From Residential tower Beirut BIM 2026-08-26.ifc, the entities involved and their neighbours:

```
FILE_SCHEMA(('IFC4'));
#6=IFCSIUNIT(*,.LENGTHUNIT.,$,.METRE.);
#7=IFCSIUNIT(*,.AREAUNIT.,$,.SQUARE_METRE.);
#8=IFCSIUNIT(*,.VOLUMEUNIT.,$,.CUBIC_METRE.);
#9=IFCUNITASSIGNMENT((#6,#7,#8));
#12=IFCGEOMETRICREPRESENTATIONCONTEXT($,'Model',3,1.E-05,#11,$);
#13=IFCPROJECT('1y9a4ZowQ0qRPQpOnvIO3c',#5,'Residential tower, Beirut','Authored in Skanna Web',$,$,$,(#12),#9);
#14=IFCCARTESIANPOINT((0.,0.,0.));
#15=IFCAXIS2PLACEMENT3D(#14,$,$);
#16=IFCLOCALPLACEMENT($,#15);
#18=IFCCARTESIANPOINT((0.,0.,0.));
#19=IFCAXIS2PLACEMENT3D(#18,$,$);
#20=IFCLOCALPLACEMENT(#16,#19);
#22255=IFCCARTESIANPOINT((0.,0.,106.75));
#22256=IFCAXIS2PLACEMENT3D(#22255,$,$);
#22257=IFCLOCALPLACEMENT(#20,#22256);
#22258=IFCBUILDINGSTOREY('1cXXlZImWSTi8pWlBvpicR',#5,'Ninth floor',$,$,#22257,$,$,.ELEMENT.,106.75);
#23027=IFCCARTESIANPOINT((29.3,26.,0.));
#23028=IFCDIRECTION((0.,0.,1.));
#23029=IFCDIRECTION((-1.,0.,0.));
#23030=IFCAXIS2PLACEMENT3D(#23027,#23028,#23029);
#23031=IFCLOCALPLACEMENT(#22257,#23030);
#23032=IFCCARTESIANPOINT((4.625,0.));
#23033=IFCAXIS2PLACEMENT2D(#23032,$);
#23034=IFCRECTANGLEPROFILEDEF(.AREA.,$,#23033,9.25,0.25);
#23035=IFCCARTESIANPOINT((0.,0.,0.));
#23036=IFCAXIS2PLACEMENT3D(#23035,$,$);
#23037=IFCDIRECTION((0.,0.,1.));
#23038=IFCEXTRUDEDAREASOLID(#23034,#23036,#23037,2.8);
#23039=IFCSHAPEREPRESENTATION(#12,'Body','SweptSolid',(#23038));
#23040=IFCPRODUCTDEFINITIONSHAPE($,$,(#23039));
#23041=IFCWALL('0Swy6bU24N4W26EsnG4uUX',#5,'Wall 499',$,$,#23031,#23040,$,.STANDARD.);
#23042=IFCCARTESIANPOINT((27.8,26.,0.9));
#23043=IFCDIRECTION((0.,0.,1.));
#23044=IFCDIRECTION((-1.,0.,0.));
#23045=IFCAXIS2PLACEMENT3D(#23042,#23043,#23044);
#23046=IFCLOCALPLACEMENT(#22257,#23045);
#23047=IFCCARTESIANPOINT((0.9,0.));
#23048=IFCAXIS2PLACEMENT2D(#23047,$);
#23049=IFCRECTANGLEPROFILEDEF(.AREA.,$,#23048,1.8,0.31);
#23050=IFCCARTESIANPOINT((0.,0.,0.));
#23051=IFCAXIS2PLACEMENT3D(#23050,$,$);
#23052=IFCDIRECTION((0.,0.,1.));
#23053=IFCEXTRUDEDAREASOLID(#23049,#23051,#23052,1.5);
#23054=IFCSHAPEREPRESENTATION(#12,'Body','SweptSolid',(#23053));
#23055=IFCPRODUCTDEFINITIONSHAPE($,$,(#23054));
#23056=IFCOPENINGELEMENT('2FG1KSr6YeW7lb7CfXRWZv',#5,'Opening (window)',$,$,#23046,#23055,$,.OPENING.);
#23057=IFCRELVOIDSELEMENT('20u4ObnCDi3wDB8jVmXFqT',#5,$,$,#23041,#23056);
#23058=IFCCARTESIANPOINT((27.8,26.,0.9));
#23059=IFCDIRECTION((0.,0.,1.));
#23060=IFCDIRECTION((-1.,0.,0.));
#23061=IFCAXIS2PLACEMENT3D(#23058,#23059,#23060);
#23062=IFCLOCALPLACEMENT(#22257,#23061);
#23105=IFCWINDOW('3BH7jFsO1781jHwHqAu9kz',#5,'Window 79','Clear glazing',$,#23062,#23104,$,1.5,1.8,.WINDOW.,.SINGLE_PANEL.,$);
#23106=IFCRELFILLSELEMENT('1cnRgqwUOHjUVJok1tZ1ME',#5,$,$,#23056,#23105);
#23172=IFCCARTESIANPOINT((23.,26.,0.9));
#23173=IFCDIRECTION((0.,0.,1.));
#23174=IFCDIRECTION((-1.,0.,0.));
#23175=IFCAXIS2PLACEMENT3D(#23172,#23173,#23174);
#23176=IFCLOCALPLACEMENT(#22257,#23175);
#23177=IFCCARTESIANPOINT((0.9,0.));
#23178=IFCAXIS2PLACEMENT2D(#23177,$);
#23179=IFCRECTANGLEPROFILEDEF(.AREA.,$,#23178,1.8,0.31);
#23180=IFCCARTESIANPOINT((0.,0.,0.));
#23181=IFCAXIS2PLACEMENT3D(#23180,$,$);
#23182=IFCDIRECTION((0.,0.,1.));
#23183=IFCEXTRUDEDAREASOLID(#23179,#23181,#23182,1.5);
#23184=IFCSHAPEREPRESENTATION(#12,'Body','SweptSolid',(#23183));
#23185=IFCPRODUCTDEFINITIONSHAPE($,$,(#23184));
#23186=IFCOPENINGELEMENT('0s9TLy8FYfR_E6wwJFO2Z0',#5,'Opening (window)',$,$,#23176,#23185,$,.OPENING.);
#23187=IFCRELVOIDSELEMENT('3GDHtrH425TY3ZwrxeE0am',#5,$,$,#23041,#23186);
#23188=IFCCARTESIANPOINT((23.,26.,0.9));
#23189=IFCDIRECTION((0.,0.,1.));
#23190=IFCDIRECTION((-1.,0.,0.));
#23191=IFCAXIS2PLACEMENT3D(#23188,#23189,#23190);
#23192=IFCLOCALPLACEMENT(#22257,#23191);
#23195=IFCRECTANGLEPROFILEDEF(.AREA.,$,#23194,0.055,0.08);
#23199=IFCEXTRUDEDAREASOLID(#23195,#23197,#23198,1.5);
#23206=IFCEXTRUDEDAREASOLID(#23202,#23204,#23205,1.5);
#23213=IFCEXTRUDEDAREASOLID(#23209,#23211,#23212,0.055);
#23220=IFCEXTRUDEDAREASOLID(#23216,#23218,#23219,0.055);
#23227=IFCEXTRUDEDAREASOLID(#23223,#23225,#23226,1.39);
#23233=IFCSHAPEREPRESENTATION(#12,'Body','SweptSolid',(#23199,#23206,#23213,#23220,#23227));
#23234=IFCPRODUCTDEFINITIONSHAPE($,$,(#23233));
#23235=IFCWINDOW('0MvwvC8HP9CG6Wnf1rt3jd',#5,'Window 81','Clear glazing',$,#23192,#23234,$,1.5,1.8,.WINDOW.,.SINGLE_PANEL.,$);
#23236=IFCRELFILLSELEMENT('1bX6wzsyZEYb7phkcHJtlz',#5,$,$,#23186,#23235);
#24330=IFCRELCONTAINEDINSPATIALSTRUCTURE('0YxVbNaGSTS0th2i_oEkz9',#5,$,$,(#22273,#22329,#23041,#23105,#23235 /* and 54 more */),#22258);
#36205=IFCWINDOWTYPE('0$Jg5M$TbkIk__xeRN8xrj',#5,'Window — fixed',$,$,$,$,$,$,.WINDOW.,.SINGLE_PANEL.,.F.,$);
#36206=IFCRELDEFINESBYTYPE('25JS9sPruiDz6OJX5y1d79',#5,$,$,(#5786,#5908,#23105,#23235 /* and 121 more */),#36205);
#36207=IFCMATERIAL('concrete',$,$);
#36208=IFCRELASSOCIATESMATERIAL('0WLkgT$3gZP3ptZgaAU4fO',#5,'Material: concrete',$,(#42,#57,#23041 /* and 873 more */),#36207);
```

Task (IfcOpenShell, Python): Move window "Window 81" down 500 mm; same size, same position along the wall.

```python
import numpy as np
import ifcopenshell
import ifcopenshell.api.geometry
import ifcopenshell.util.placement
import ifcopenshell.util.unit

model = ifcopenshell.open("Residential tower Beirut BIM 2026-08-26.ifc")
unit_scale = ifcopenshell.util.unit.calculate_unit_scale(model)

window = model.by_guid("0MvwvC8HP9CG6Wnf1rt3jd")
opening = window.FillsVoids[0].RelatingOpeningElement
dz = -0.5

shift = np.array([0.0, 0.0, dz])
# The window is not placed relative to its opening, so move both.
for product in (opening, window):
    matrix = ifcopenshell.util.placement.get_local_placement(product.ObjectPlacement)
    matrix[:3, 3] += shift
    ifcopenshell.api.geometry.edit_object_placement(model, product=product, matrix=matrix, is_si=False)

print(f"moved by {dz * unit_scale:+.3f} m")

model.write("Residential tower Beirut BIM 2026-08-26_v2.ifc")
```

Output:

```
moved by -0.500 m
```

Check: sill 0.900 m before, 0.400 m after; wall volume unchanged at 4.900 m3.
